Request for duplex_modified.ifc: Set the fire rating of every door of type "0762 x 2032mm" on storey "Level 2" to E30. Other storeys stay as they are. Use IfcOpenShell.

First a look at what the model holds.

```python
import ifcopenshell
import ifcopenshell.util.element

model = ifcopenshell.open("duplex_modified.ifc")
print(model.schema)
storey = next(s for s in model.by_type("IfcBuildingStorey") if s.Name == "Level 2")
doors = [e for e in ifcopenshell.util.element.get_decomposition(storey) if e.is_a("IfcDoor")]
seen = {}
for e in doors:
    element_type = ifcopenshell.util.element.get_type(e)
    key = (element_type.Name if element_type != e and element_type else None, ifcopenshell.util.element.get_pset(e, "Pset_DoorCommon", "FireRating"))
    seen[key] = seen.get(key, 0) + 1
for (name, value), count in sorted(seen.items(), key=str):
    print(count, "x", name, "|", value)
```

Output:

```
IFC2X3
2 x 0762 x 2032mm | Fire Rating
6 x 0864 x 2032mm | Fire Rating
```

```python
import ifcopenshell
import ifcopenshell.api.pset
import ifcopenshell.util.element

model = ifcopenshell.open("duplex_modified.ifc")

storey = next(s for s in model.by_type("IfcBuildingStorey") if s.Name == "Level 2")
doors = [e for e in ifcopenshell.util.element.get_decomposition(storey) if e.is_a("IfcDoor")]

count = 0
for e in doors:
    element_type = ifcopenshell.util.element.get_type(e)
    if element_type in (None, e) or element_type.Name != "0762 x 2032mm":
        continue
    # add_pset returns the element's existing set when there is one.
    pset = ifcopenshell.api.pset.add_pset(model, product=e, name="Pset_DoorCommon")
    ifcopenshell.api.pset.edit_pset(model, pset=pset, properties={"FireRating": "E30"})
    count += 1

print(count, "doors updated")

model.write("duplex_modified_rev.ifc")
```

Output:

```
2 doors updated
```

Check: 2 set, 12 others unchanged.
